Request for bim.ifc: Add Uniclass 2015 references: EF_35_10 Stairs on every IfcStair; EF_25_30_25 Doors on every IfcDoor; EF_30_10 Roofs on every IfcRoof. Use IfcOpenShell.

First a look at what the model holds.

```python
import ifcopenshell

model = ifcopenshell.open("bim.ifc")
print(model.schema)
print("classifications:", [c.Name for c in model.by_type("IfcClassification")])
for ifc_class in ("IfcDoor", "IfcRoof", "IfcStair", "IfcWall", "IfcWindow"):
    print(ifc_class, len(model.by_type(ifc_class)))
```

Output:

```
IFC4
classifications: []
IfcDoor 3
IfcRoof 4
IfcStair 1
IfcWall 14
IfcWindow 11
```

```python
import ifcopenshell
import ifcopenshell.api.classification

model = ifcopenshell.open("bim.ifc")

system = ifcopenshell.api.classification.add_classification(model, classification="Uniclass 2015")

codes = {
    "IfcStair": ("EF_35_10", "Stairs"),
    "IfcDoor": ("EF_25_30_25", "Doors"),
    "IfcRoof": ("EF_30_10", "Roofs"),
}
for ifc_class, (code, name) in codes.items():
    products = model.by_type(ifc_class)
    ifcopenshell.api.classification.add_reference(
        model, products=products, classification=system, identification=code, name=name
    )
    print(code, len(products))

model.write("bim_edited.ifc")
```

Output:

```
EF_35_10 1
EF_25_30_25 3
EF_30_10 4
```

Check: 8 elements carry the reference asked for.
